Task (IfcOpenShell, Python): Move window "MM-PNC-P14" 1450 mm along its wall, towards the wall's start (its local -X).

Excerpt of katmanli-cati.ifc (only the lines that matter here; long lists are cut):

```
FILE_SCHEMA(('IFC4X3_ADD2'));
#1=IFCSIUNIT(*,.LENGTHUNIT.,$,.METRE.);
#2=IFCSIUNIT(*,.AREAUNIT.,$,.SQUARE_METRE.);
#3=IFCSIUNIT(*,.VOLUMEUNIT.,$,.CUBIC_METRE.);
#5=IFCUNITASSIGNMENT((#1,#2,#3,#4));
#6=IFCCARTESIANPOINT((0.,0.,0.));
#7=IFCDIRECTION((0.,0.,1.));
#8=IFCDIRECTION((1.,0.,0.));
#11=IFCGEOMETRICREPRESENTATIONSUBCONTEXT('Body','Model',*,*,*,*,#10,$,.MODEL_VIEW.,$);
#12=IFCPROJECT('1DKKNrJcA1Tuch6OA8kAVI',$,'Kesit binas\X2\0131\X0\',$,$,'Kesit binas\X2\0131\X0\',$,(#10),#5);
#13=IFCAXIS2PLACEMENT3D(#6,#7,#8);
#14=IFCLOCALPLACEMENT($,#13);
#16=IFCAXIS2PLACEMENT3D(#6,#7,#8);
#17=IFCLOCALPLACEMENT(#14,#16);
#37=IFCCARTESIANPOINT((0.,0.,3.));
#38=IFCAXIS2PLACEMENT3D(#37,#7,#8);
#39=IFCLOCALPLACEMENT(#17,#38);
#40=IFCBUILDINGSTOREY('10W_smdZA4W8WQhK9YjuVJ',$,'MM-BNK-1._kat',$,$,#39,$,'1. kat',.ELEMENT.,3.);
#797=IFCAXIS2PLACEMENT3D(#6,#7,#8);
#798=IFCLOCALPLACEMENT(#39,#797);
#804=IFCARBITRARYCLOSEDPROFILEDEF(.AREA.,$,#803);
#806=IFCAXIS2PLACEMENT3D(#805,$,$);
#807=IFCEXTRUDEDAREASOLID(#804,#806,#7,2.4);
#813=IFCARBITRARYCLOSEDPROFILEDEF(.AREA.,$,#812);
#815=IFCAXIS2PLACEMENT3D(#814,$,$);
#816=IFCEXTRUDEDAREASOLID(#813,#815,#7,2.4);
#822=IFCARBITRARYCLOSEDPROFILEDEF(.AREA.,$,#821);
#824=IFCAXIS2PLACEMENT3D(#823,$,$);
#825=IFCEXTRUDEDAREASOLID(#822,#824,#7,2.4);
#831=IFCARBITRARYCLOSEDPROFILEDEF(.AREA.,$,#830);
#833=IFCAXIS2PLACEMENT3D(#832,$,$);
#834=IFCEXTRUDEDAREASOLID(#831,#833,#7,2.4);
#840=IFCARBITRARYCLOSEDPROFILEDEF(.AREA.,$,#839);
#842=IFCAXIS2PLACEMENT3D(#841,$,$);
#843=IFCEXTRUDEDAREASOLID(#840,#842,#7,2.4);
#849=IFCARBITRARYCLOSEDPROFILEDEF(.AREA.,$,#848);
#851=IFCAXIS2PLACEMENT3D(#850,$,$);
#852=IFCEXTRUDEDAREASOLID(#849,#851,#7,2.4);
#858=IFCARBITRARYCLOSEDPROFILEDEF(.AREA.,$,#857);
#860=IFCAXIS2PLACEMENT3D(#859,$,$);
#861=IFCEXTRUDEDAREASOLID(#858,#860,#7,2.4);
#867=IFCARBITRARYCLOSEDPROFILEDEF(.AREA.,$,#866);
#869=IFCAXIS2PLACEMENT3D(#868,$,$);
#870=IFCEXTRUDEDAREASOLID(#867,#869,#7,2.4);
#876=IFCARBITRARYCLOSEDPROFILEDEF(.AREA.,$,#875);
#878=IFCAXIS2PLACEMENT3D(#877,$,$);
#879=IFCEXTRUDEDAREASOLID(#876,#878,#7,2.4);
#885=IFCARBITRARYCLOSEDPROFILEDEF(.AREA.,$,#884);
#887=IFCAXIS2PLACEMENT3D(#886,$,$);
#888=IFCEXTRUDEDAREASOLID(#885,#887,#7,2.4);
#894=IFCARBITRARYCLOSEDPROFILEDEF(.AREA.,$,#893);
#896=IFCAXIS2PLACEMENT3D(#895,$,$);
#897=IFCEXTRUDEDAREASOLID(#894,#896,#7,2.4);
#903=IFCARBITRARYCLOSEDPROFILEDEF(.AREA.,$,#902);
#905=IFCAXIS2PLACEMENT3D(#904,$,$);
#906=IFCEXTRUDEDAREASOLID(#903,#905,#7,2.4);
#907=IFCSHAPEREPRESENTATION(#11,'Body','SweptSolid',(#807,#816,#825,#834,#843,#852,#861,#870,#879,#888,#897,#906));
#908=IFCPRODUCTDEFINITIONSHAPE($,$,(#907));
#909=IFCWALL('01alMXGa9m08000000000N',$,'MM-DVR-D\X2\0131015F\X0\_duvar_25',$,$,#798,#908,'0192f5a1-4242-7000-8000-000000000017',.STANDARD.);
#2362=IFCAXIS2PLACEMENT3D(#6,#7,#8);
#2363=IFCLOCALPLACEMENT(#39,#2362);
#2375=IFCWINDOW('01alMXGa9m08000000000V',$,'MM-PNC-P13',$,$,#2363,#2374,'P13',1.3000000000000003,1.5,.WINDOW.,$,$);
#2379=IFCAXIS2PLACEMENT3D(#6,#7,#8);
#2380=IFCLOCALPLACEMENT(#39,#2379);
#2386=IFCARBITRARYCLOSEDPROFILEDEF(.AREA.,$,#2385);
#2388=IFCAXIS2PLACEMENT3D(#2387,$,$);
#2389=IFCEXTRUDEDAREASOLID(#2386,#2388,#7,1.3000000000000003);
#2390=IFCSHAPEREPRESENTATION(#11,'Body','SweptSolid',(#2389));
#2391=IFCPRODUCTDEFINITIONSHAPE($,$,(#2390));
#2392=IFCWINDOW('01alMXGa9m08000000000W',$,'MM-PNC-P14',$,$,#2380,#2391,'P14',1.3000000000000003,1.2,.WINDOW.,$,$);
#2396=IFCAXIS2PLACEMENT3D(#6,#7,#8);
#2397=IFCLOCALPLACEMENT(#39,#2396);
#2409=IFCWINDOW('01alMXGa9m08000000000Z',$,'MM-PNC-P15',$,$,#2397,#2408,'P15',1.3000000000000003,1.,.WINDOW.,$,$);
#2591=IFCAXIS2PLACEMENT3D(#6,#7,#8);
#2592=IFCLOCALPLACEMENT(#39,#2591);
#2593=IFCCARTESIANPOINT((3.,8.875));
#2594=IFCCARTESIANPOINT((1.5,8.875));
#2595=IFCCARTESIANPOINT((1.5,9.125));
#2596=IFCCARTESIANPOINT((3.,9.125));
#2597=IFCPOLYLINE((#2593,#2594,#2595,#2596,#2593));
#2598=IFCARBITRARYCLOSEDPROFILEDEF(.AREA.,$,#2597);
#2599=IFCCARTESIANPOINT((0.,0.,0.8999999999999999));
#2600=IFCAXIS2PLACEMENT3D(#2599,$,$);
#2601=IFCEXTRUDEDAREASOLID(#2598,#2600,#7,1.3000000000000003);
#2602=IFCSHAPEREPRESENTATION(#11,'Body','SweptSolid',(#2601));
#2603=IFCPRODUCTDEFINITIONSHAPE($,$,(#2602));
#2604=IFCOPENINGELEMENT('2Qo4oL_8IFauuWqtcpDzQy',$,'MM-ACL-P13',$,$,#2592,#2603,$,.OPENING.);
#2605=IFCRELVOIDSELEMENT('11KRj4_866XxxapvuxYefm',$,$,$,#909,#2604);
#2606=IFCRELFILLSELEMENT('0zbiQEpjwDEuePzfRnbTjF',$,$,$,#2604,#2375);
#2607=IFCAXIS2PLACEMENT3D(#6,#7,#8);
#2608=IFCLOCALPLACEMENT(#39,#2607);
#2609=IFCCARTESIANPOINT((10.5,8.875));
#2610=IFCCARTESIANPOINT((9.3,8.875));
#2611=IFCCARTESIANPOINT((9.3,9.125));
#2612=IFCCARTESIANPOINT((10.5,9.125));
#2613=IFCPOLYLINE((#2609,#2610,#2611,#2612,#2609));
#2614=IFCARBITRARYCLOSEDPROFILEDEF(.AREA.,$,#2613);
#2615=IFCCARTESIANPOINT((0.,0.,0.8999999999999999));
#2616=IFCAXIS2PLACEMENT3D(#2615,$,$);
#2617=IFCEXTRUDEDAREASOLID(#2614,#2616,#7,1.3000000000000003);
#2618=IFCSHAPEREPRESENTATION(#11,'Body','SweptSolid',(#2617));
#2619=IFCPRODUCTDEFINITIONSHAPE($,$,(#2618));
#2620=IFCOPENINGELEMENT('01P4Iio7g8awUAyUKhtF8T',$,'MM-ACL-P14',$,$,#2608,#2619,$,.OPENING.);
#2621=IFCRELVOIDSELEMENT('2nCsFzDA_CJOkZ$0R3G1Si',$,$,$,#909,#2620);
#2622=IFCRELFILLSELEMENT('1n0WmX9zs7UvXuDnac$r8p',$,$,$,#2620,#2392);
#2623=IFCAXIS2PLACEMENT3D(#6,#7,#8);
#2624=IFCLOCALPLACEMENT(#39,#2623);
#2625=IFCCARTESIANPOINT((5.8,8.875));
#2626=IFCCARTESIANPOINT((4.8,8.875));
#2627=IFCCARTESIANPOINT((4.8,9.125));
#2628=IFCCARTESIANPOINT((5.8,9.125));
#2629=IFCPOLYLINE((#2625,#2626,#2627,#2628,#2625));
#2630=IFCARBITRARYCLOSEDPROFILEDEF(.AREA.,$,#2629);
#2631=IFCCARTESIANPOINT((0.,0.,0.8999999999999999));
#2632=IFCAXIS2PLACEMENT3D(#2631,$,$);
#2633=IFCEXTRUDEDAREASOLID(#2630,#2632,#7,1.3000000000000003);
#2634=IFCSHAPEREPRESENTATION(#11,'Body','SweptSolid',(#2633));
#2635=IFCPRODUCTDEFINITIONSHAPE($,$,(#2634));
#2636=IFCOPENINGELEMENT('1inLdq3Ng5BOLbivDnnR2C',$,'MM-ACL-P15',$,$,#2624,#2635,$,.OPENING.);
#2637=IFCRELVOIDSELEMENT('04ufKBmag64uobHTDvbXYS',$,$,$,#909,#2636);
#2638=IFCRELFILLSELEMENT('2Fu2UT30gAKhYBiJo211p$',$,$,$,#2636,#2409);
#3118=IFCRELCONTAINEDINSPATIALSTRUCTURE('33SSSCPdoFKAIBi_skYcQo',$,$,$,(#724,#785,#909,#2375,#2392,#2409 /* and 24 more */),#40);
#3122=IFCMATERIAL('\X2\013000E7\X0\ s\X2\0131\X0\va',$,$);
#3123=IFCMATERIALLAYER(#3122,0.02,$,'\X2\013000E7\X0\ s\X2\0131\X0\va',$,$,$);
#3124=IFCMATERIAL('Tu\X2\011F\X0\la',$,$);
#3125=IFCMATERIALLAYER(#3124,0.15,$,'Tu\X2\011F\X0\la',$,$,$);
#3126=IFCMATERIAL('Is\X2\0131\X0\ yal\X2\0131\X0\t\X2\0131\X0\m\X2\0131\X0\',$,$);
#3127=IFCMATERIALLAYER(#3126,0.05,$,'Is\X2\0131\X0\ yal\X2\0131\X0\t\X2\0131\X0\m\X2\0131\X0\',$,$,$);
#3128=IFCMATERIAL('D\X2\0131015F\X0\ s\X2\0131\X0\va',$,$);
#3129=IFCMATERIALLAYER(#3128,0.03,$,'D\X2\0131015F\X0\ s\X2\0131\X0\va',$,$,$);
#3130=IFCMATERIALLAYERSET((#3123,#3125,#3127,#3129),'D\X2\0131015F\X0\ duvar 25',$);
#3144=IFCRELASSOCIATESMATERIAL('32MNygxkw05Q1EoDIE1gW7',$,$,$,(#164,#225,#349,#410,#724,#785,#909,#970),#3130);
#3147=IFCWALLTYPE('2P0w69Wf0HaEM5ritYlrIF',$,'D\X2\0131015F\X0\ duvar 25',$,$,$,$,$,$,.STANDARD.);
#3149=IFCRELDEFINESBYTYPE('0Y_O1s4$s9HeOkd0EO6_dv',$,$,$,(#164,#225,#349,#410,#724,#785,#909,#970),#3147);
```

```python
import ifcopenshell
import ifcopenshell.api.geometry
import ifcopenshell.util.placement

model = ifcopenshell.open("katmanli-cati.ifc")

window = model.by_guid("01alMXGa9m08000000000W")
opening = window.FillsVoids[0].RelatingOpeningElement
wall = opening.VoidsElements[0].RelatingBuildingElement

wall_matrix = ifcopenshell.util.placement.get_local_placement(wall.ObjectPlacement)
shift = wall_matrix[:3, 0] * -1.45
before = ifcopenshell.util.placement.get_local_placement(window.ObjectPlacement)[:3, 3].copy()

# The window is not placed relative to its opening, so move both.
for product in (opening, window):
    matrix = ifcopenshell.util.placement.get_local_placement(product.ObjectPlacement)
    matrix[:3, 3] += shift
    ifcopenshell.api.geometry.edit_object_placement(model, product=product, matrix=matrix, is_si=False)

after = ifcopenshell.util.placement.get_local_placement(window.ObjectPlacement)[:3, 3]
print("window moved by", (after - before).round(3) + 0.0)

model.write("katmanli-cati-out.ifc")
```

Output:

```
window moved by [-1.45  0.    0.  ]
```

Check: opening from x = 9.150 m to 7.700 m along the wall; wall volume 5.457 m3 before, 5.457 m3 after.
